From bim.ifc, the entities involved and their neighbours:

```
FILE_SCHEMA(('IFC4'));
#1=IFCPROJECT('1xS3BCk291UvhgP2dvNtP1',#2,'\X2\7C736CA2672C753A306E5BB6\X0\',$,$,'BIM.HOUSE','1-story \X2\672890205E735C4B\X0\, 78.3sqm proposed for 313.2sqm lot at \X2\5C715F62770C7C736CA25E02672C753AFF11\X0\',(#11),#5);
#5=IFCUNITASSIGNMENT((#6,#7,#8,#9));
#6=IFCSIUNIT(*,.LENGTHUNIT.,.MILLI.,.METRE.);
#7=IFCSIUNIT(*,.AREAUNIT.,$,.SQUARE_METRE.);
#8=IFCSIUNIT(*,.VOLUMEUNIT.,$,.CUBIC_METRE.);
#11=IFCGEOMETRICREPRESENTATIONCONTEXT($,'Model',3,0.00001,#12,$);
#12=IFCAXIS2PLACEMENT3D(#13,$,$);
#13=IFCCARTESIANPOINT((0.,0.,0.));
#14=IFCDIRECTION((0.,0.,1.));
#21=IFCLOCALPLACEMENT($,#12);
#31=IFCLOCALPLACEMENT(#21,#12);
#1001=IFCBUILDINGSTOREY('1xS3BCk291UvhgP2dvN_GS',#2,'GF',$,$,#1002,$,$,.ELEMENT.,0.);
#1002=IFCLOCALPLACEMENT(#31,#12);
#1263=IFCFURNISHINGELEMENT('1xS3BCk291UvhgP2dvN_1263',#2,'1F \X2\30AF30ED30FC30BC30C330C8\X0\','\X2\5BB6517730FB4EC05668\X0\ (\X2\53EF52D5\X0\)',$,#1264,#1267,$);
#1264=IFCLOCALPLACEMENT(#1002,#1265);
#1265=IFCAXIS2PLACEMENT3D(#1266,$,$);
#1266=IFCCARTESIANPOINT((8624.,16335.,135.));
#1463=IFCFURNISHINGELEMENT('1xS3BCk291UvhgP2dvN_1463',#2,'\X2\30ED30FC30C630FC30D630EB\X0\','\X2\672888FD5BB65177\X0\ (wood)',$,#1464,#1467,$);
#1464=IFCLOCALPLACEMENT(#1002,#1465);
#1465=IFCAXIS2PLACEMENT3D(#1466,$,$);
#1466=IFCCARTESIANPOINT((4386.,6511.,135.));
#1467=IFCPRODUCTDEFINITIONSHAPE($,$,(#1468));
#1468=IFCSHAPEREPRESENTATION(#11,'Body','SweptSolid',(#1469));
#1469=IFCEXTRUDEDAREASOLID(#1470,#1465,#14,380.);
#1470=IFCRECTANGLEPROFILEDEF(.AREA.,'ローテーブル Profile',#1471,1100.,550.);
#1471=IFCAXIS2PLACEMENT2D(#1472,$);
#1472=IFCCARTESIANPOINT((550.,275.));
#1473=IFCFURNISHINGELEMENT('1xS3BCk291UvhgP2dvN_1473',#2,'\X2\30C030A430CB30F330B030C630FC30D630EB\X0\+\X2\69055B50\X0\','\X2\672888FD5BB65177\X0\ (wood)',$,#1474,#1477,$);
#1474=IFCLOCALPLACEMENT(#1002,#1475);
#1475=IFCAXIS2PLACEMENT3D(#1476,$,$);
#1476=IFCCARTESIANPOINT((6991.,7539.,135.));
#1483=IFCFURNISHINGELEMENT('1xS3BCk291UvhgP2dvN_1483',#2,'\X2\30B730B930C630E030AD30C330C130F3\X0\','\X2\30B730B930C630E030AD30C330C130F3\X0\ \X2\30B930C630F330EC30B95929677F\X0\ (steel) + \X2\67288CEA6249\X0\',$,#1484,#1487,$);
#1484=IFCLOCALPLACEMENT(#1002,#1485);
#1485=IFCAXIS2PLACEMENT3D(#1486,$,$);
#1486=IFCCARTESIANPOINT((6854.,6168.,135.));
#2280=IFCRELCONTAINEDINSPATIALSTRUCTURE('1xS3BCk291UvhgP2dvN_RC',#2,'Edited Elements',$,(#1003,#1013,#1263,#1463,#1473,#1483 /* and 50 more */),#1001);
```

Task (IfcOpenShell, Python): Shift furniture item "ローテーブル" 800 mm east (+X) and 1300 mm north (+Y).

```python
import ifcopenshell
import ifcopenshell.api.geometry
import ifcopenshell.util.placement
import ifcopenshell.util.unit

model = ifcopenshell.open("bim.ifc")
unit_scale = ifcopenshell.util.unit.calculate_unit_scale(model)

item = model.by_guid("1xS3BCk291UvhgP2dvN_1463")
matrix = ifcopenshell.util.placement.get_local_placement(item.ObjectPlacement)
matrix[0, 3] += 0.8 / unit_scale
matrix[1, 3] += 1.3 / unit_scale
ifcopenshell.api.geometry.edit_object_placement(model, product=item, matrix=matrix, is_si=False)

print(ifcopenshell.util.placement.get_local_placement(item.ObjectPlacement).round(3) + 0.0)

model.write("bim-out.ifc")
```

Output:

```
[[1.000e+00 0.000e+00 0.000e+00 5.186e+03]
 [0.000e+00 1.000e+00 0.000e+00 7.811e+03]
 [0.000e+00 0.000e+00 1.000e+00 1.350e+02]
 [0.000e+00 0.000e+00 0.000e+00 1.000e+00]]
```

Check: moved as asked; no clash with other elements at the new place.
